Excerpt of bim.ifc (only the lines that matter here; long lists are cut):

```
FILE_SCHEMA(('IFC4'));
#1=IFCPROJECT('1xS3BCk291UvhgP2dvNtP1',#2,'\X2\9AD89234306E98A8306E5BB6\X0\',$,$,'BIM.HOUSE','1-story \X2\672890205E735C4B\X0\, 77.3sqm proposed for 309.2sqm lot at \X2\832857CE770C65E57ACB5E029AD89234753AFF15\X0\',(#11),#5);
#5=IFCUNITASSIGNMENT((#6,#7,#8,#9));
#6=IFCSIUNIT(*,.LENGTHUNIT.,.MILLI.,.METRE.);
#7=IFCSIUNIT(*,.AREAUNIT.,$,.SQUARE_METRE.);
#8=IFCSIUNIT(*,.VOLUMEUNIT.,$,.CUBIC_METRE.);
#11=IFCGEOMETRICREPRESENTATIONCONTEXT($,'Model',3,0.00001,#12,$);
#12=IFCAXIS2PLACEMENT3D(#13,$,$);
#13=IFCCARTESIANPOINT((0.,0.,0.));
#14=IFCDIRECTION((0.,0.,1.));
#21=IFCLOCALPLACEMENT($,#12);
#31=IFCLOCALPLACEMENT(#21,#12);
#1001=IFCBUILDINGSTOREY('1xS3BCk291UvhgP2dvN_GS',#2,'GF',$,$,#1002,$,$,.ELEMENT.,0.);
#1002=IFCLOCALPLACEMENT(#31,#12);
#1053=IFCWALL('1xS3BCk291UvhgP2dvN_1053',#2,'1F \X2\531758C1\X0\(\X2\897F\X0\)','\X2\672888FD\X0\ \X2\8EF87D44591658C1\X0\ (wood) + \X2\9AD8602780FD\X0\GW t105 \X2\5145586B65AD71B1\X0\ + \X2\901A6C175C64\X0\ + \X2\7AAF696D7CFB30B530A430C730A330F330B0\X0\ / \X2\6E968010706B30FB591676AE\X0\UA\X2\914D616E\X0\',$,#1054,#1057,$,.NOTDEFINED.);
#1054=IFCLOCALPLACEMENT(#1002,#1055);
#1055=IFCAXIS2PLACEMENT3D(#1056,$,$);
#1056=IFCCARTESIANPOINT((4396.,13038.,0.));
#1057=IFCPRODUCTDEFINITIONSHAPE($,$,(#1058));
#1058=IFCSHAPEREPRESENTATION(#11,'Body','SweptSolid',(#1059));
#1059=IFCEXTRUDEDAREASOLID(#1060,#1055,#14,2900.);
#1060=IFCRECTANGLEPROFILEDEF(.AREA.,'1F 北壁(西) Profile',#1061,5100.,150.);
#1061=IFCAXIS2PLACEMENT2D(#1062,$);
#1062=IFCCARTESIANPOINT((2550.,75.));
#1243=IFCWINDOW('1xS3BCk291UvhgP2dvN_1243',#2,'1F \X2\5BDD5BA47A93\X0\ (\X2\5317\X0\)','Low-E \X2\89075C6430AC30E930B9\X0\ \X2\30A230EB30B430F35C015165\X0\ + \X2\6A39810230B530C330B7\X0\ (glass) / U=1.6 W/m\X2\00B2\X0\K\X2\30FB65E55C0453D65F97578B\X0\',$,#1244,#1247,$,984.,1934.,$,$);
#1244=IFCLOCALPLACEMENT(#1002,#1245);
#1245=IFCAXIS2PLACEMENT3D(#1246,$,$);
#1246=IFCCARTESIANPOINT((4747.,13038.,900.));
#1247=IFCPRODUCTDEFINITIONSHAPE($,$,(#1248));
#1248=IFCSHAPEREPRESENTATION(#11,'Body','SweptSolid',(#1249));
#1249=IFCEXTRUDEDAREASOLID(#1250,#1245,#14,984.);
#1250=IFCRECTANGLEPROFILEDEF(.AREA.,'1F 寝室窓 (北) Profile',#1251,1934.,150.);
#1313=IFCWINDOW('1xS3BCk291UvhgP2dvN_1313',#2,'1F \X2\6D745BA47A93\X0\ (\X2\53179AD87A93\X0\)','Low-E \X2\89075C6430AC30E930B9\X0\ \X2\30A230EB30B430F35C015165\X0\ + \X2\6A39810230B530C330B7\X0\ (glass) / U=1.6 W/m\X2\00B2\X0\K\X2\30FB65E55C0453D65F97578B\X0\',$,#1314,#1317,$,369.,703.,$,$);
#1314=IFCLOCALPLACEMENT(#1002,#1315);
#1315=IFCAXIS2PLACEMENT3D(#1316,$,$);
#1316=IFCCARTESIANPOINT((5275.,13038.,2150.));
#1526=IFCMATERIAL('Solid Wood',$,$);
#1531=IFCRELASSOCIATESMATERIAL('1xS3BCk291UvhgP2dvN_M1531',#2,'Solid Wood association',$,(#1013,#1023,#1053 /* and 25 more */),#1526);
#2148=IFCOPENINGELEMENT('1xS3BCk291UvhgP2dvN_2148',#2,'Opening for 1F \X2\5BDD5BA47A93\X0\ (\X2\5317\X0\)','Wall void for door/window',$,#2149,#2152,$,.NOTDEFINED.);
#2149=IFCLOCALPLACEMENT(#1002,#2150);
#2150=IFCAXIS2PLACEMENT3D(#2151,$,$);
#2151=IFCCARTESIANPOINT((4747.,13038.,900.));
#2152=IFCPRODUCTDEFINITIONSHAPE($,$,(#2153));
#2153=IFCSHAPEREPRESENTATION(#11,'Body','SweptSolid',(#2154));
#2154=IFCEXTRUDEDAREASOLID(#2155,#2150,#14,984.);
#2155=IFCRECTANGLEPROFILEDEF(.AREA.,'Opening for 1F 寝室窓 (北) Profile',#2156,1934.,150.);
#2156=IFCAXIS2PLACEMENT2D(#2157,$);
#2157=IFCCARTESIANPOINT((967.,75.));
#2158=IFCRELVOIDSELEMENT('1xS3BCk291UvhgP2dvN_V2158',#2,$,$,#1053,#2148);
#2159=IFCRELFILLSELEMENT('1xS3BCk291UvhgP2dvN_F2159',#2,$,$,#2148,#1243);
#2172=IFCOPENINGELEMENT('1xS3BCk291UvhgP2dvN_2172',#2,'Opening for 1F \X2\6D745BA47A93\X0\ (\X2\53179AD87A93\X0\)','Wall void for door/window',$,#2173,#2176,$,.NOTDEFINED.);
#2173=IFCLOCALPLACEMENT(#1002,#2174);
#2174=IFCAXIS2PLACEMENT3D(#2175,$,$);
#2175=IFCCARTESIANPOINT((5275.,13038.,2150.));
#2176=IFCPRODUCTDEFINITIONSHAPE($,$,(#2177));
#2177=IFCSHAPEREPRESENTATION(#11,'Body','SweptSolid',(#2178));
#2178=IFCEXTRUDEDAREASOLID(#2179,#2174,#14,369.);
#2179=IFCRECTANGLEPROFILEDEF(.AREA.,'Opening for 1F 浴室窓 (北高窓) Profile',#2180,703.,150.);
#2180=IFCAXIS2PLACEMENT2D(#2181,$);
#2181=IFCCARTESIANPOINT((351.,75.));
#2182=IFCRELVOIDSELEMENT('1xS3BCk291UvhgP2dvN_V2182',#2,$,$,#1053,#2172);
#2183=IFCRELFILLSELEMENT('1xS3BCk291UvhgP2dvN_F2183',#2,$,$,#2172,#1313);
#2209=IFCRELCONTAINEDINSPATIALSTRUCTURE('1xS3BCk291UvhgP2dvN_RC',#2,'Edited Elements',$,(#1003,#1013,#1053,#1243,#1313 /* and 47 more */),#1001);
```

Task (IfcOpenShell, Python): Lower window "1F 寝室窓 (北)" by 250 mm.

```python
import numpy as np
import ifcopenshell
import ifcopenshell.api.geometry
import ifcopenshell.util.placement
import ifcopenshell.util.unit

model = ifcopenshell.open("bim.ifc")
unit_scale = ifcopenshell.util.unit.calculate_unit_scale(model)

window = model.by_guid("1xS3BCk291UvhgP2dvN_1243")
opening = window.FillsVoids[0].RelatingOpeningElement
dz = -0.25 / unit_scale

shift = np.array([0.0, 0.0, dz])
# The window is not placed relative to its opening, so move both.
for product in (opening, window):
    matrix = ifcopenshell.util.placement.get_local_placement(product.ObjectPlacement)
    matrix[:3, 3] += shift
    ifcopenshell.api.geometry.edit_object_placement(model, product=product, matrix=matrix, is_si=False)

print(f"moved by {dz * unit_scale:+.3f} m")

model.write("bim-out.ifc")
```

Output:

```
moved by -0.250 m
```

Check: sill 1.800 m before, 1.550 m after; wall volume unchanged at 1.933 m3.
